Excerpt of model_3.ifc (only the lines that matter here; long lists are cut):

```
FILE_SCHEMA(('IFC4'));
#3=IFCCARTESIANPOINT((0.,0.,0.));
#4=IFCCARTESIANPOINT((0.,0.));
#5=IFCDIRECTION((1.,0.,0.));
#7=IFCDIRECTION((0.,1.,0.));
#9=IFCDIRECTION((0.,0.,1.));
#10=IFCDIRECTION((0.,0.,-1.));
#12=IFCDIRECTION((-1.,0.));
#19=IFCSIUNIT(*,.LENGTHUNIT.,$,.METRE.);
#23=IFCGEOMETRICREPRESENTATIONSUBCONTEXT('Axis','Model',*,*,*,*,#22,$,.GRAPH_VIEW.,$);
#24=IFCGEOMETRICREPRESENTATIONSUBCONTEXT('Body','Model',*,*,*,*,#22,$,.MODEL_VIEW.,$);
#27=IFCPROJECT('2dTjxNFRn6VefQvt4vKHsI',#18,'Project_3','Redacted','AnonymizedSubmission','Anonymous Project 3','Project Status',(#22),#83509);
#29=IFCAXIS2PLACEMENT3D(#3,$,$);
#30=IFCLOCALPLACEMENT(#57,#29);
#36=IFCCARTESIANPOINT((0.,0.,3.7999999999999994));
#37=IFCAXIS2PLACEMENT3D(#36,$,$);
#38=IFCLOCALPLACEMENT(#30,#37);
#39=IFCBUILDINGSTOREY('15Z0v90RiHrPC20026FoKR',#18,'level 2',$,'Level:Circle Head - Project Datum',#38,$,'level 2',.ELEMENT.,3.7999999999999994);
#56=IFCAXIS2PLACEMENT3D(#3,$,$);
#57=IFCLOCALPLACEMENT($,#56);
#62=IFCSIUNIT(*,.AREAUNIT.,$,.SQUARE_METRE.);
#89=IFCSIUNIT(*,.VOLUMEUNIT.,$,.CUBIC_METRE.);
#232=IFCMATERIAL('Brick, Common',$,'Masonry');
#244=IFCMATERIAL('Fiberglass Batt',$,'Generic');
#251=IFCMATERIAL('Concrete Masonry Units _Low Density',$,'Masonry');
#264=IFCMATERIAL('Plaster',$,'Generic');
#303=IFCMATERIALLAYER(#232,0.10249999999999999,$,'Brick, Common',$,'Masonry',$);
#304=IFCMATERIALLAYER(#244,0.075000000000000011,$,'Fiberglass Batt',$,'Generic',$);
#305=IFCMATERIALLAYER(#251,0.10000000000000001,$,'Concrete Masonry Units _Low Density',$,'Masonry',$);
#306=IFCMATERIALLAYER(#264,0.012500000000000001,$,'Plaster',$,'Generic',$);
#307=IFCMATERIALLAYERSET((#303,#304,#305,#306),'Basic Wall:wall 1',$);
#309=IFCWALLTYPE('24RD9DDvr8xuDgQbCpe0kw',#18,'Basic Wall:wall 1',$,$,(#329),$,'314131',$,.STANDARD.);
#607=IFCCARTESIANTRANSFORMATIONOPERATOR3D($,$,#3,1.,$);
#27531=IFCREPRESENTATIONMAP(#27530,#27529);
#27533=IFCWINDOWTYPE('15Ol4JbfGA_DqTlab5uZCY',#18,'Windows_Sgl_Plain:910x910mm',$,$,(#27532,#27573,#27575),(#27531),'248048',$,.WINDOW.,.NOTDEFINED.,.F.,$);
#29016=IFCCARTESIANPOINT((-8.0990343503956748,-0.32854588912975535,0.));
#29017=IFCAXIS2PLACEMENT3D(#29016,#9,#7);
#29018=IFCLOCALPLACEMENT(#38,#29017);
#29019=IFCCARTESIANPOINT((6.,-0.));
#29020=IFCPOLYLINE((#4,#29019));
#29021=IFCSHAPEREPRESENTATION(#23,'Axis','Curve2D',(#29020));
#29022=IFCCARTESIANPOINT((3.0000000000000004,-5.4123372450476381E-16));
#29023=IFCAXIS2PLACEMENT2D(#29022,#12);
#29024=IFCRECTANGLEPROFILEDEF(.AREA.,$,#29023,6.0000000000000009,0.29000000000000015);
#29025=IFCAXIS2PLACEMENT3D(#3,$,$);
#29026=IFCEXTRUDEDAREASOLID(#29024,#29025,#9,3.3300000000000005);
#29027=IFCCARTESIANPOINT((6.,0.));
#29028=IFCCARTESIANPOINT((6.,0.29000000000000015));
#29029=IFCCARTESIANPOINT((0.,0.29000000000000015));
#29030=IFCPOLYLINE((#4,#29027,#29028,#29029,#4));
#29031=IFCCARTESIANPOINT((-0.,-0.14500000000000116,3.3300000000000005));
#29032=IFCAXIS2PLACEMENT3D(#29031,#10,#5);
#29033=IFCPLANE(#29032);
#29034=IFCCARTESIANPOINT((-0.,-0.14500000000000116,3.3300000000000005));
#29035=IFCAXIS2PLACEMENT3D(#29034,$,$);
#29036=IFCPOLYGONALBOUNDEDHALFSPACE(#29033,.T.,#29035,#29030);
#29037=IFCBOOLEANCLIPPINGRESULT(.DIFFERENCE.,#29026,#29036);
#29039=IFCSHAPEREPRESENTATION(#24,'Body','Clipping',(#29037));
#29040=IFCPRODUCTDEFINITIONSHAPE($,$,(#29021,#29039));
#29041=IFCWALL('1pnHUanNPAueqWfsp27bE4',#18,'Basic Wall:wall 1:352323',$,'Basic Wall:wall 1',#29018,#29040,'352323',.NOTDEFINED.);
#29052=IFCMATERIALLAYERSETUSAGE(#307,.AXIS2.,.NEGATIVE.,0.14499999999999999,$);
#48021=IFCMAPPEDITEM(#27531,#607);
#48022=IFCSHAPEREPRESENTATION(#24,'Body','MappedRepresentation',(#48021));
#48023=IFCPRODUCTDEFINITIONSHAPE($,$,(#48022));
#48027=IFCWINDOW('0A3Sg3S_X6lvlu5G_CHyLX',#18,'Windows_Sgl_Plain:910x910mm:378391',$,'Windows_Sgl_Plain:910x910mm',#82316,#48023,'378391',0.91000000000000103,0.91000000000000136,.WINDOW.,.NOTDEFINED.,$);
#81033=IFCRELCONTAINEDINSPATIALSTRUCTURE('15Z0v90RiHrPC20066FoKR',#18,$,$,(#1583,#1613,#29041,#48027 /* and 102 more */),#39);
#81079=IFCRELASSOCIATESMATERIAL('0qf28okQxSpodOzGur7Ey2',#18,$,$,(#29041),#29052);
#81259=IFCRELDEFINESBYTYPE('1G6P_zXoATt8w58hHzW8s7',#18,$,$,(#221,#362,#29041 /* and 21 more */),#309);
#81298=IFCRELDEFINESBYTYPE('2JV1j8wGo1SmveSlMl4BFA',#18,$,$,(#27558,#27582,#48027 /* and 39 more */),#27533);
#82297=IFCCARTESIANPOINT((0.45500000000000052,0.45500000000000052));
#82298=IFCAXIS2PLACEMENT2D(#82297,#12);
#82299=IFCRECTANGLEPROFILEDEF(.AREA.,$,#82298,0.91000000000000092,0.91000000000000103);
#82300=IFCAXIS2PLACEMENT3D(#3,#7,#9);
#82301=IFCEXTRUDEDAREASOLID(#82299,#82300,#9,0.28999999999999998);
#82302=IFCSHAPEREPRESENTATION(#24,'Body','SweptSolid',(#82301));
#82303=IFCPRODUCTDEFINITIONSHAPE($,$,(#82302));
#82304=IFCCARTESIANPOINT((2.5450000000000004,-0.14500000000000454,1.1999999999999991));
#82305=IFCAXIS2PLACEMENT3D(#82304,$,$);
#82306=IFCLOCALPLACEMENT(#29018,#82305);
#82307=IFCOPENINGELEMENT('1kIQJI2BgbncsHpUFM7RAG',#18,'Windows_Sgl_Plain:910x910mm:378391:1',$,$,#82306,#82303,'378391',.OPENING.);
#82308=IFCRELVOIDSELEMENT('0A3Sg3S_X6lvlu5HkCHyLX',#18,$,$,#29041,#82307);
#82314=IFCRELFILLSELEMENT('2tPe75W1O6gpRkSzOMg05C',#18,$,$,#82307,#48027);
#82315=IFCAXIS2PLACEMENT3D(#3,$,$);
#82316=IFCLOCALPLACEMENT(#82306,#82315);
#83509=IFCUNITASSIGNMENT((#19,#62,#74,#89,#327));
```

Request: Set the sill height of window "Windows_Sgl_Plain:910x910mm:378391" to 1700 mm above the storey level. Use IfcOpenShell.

```python
import numpy as np
import ifcopenshell
import ifcopenshell.api.geometry
import ifcopenshell.geom
import ifcopenshell.util.element
import ifcopenshell.util.placement
import ifcopenshell.util.shape
import ifcopenshell.util.unit

model = ifcopenshell.open("model_3.ifc")
unit_scale = ifcopenshell.util.unit.calculate_unit_scale(model)

window = model.by_guid("0A3Sg3S_X6lvlu5G_CHyLX")
opening = window.FillsVoids[0].RelatingOpeningElement
storey = ifcopenshell.util.element.get_container(window, ifc_class="IfcBuildingStorey")
level = ifcopenshell.util.placement.get_local_placement(storey.ObjectPlacement)[2, 3]

# The opening's origin need not be at the sill, so measure its lowest point.
shape = ifcopenshell.geom.create_shape(ifcopenshell.geom.settings(), opening)
bottom = ifcopenshell.util.shape.get_shape_bottom_elevation(shape, shape.geometry) / unit_scale
dz = level + 1.7 - bottom

shift = np.array([0.0, 0.0, dz])
# The window is placed relative to its opening, so it follows when the opening moves.
matrix = ifcopenshell.util.placement.get_local_placement(opening.ObjectPlacement)
matrix[:3, 3] += shift
ifcopenshell.api.geometry.edit_object_placement(
    model, product=opening, matrix=matrix, is_si=False, should_transform_children=True
)

print(f"moved by {dz * unit_scale:+.3f} m")

model.write("model_3-out.ifc")
```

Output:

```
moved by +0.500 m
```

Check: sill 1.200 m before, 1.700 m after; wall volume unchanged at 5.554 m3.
